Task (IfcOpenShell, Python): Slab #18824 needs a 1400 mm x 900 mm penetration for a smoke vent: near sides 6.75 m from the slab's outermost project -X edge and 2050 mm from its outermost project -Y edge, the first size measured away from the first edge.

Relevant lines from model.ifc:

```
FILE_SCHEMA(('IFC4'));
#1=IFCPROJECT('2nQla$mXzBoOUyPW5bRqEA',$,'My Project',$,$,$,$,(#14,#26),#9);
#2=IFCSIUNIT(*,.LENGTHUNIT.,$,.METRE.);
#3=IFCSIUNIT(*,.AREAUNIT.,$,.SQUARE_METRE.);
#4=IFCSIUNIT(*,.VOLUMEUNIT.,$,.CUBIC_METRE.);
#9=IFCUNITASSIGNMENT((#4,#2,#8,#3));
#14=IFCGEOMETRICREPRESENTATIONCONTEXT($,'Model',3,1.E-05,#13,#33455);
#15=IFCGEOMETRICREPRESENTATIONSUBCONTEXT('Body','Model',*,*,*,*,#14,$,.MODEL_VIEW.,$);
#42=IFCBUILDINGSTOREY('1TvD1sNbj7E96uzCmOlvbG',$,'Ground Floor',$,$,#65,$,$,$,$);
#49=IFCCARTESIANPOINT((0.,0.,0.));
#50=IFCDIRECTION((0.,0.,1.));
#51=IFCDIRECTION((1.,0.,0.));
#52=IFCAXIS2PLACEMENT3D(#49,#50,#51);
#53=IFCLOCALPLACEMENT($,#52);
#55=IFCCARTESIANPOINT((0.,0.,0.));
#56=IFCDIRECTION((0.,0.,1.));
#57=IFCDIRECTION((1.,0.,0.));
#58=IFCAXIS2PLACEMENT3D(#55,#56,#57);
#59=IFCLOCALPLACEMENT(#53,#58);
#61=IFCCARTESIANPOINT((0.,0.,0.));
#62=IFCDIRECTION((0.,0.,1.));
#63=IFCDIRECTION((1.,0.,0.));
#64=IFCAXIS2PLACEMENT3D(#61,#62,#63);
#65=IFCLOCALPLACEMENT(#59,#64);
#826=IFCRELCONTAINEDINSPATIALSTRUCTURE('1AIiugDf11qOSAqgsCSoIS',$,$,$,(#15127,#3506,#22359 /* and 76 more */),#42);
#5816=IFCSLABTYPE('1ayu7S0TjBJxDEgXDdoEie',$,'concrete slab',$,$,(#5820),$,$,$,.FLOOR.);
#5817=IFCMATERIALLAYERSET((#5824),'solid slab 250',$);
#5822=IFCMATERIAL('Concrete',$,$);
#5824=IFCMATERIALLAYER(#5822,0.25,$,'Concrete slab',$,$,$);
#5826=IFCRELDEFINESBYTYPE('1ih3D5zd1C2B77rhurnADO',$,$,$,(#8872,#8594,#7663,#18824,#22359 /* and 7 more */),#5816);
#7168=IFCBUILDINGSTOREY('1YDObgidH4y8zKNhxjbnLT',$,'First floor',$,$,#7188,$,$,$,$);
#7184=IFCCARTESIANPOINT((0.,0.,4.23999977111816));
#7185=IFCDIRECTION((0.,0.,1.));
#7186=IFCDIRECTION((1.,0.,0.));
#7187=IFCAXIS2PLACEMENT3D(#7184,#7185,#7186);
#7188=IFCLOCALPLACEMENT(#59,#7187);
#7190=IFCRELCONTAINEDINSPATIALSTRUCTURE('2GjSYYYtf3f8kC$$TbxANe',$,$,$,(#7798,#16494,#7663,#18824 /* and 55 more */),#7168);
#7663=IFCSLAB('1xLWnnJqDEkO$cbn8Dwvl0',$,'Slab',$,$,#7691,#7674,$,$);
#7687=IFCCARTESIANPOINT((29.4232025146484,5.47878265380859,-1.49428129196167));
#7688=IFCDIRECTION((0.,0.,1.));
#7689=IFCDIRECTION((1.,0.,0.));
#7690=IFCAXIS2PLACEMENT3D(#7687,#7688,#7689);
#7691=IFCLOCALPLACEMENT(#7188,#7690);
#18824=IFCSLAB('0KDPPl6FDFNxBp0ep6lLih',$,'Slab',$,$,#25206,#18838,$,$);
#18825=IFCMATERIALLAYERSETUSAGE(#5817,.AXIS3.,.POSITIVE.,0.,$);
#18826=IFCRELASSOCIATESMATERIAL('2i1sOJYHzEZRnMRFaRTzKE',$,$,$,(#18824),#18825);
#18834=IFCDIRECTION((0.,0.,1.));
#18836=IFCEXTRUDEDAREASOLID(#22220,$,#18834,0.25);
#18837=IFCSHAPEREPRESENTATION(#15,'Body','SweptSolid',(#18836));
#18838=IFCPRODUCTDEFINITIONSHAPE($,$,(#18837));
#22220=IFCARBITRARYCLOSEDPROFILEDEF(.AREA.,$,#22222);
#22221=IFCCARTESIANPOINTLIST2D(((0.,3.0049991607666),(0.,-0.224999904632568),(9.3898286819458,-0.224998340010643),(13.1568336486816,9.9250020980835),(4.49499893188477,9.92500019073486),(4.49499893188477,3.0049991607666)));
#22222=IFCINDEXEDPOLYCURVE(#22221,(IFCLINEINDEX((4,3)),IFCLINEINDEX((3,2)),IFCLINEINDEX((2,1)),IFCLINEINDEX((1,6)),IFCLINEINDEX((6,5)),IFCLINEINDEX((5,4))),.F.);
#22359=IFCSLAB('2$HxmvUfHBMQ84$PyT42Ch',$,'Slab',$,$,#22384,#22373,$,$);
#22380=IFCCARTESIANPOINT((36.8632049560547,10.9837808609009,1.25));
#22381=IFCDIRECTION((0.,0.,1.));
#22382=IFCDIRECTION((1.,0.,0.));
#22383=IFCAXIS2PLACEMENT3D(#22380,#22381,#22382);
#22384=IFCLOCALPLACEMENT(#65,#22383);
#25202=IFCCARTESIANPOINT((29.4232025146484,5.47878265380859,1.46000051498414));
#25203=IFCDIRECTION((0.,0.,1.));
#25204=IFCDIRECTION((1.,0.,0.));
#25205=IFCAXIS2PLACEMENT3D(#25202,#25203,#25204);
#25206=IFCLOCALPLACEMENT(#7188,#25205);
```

```python
import numpy as np
import ifcopenshell
import ifcopenshell.api.feature
import ifcopenshell.api.geometry
import ifcopenshell.api.root
import ifcopenshell.geom
import ifcopenshell.util.placement
import ifcopenshell.util.representation
import ifcopenshell.util.shape
import ifcopenshell.util.unit

model = ifcopenshell.open("model.ifc")
unit_scale = ifcopenshell.util.unit.calculate_unit_scale(model)
settings = ifcopenshell.geom.settings()


def volume(element):
    """Net volume in cubic metres, openings subtracted."""
    shape = ifcopenshell.geom.create_shape(settings, element)
    return ifcopenshell.util.shape.get_volume(shape.geometry)


slab = model.by_guid("0KDPPl6FDFNxBp0ep6lLih")
before = volume(slab)

# Extent in the slab's own axes, in metres. The edges named are its -X and -Y sides.
slab_shape = ifcopenshell.geom.create_shape(settings, slab)
vertices = ifcopenshell.util.shape.get_vertices(slab_shape.geometry)
x_min, y_min, bottom = vertices.min(axis=0)
top = vertices[:, 2].max()

opening = ifcopenshell.api.root.create_entity(model, ifc_class="IfcOpeningElement", name="Smoke vent opening", predefined_type="OPENING")
context = ifcopenshell.util.representation.get_context(model, "Model", "Body", "MODEL_VIEW")
width, depth = 1.4, 0.9
outline = [(0.0, 0.0), (width, 0.0), (width, depth), (0.0, depth), (0.0, 0.0)]
# Overshoot both faces by 50 mm so the cut is clean.
shape = ifcopenshell.api.geometry.add_slab_representation(
    model, context=context, depth=top - bottom + 0.1, polyline=outline
)
ifcopenshell.api.geometry.assign_representation(model, product=opening, representation=shape)

matrix = ifcopenshell.util.placement.get_local_placement(slab.ObjectPlacement)
matrix[:, 3] = matrix @ np.append(np.array([x_min + 6.75, y_min + 2.05, bottom - 0.05]) / unit_scale, 1.0)
ifcopenshell.api.geometry.edit_object_placement(model, product=opening, matrix=matrix, is_si=False)
ifcopenshell.api.feature.add_feature(model, feature=opening, element=slab)

after = volume(slab)

print(f"slab volume {before:.3f} -> {after:.3f} m3")

model.write("model_edited.ifc")
```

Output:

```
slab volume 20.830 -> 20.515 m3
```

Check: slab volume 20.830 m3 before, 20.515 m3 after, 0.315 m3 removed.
